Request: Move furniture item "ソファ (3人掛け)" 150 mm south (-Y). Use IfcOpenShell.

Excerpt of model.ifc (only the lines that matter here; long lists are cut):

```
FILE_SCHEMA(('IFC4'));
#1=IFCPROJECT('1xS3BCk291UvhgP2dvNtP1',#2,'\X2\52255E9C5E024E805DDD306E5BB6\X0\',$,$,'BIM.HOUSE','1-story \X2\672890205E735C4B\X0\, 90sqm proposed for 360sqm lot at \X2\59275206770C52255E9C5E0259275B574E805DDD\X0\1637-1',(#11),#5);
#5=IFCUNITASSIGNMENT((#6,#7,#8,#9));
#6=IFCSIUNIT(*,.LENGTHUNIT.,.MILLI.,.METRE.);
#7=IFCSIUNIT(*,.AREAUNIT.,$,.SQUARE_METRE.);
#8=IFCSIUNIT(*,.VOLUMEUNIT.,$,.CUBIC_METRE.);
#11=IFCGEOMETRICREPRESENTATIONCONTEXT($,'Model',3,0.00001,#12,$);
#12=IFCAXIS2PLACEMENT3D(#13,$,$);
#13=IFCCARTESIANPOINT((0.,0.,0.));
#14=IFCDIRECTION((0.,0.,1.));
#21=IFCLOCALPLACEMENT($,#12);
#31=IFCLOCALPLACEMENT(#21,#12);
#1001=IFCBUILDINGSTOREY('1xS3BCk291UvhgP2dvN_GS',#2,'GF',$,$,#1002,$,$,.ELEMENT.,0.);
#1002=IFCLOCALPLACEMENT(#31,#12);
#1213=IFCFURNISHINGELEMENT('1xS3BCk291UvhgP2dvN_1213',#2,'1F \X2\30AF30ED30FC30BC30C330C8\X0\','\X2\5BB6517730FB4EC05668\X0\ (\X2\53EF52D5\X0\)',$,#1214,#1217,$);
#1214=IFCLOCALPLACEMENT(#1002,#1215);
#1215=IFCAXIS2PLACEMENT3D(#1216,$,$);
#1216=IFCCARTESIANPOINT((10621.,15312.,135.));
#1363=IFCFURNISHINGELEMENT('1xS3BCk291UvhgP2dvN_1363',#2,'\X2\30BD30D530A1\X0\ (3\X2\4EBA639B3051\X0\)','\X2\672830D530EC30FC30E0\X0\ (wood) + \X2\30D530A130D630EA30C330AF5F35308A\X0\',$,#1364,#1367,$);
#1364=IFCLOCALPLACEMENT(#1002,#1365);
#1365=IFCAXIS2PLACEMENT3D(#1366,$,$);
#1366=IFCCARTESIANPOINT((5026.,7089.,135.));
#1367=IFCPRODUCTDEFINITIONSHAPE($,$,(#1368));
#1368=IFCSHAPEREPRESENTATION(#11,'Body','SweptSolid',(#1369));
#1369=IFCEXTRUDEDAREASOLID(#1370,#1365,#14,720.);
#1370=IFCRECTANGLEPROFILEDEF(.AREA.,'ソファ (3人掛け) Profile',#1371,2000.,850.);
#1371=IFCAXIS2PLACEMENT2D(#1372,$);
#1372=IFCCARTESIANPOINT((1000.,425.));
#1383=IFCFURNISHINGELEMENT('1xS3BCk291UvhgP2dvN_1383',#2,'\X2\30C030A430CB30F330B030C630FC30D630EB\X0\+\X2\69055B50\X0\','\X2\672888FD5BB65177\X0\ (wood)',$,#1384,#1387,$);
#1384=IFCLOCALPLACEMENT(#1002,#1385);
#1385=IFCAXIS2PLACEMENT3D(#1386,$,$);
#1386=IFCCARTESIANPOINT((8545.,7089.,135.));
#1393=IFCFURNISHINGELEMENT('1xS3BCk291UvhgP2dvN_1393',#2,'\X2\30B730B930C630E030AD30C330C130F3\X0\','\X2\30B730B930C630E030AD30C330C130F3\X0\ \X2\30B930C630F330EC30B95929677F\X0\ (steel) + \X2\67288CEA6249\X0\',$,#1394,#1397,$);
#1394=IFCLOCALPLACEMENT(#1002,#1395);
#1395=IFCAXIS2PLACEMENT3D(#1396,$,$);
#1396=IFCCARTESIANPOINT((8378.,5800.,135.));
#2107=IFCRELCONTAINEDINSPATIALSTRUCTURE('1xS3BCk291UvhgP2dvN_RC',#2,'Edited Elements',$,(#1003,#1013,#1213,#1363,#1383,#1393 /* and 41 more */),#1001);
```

```python
import ifcopenshell
import ifcopenshell.api.geometry
import ifcopenshell.util.placement
import ifcopenshell.util.unit

model = ifcopenshell.open("model.ifc")
unit_scale = ifcopenshell.util.unit.calculate_unit_scale(model)

item = model.by_id(1363)
matrix = ifcopenshell.util.placement.get_local_placement(item.ObjectPlacement)
matrix[1, 3] -= 0.15 / unit_scale
ifcopenshell.api.geometry.edit_object_placement(model, product=item, matrix=matrix, is_si=False)

print(ifcopenshell.util.placement.get_local_placement(item.ObjectPlacement).round(3) + 0.0)

model.write("model_rev.ifc")
```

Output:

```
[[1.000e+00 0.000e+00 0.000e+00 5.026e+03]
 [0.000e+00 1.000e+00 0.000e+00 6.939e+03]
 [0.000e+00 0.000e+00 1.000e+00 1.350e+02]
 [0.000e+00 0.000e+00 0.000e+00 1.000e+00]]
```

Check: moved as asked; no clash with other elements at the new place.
